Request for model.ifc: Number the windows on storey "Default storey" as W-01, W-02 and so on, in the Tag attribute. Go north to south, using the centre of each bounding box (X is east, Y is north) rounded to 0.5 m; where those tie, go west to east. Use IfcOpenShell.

First a look at what the model holds.

```python
import ifcopenshell
import ifcopenshell.util.element
import ifcopenshell.util.placement

model = ifcopenshell.open("model.ifc")
print(model.schema)
storey = next(s for s in model.by_type("IfcBuildingStorey") if s.Name == "Default storey")
windows = [e for e in ifcopenshell.util.element.get_decomposition(storey) if e.is_a("IfcWindow")]
for e in sorted(windows, key=lambda e: e.id()):
    origin = ifcopenshell.util.placement.get_local_placement(e.ObjectPlacement)[:3, 3]
    print(e.id(), e.Tag, e.Name, origin.round(2) + 0.0, sep=" | ")
```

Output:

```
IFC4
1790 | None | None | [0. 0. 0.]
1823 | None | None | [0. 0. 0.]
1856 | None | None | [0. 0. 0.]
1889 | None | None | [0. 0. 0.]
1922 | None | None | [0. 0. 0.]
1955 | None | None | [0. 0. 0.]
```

```python
import ifcopenshell
import ifcopenshell.geom
import ifcopenshell.util.element
import ifcopenshell.util.shape

model = ifcopenshell.open("model.ifc")
settings = ifcopenshell.geom.settings()
settings.set("use-world-coords", True)


def centre(element):
    shape = ifcopenshell.geom.create_shape(settings, element)
    return ifcopenshell.util.shape.get_bbox_centroid(shape.geometry)


storey = next(s for s in model.by_type("IfcBuildingStorey") if s.Name == "Default storey")
windows = [e for e in ifcopenshell.util.element.get_decomposition(storey) if e.is_a("IfcWindow")]

# Insertion points can sit at a corner or the storey origin, so sort by the geometry (in metres).
centres = {e: centre(e) for e in windows}
windows.sort(key=lambda e: (-round(centres[e][1] / 0.5), centres[e][0]))

for i, e in enumerate(windows, start=1):
    number = f"W-{i:02d}"
    e.Tag = number
    print(e.id(), number)

model.write("model-out.ifc")
```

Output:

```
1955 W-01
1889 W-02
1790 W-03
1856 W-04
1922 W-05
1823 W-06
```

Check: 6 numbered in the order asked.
